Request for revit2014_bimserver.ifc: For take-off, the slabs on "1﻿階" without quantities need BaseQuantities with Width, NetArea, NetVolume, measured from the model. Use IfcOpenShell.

First a look at what the model holds.

```python
import ifcopenshell
import ifcopenshell.util.element
import ifcopenshell.util.unit

model = ifcopenshell.open("revit2014_bimserver.ifc")
print(model.schema)
for unit_type in ("LENGTHUNIT", "AREAUNIT", "VOLUMEUNIT"):
    print(unit_type, ifcopenshell.util.unit.calculate_unit_scale(model, unit_type))
storey = next(s for s in model.by_type("IfcBuildingStorey") if s.Name == '1\ufeff階')
slabs = [e for e in ifcopenshell.util.element.get_decomposition(storey) if e.is_a("IfcSlab")]
for e in sorted(slabs, key=lambda e: e.id()):
    print(e.id(), e.is_a(), e.Name, list(ifcopenshell.util.element.get_psets(e, qtos_only=True)), sep=" | ")
```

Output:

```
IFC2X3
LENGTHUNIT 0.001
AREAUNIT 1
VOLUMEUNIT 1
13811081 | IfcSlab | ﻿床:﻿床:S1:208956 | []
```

```python
import ifcopenshell
import ifcopenshell.api.pset
import ifcopenshell.geom
import ifcopenshell.util.element
import ifcopenshell.util.shape
import ifcopenshell.util.unit

model = ifcopenshell.open("revit2014_bimserver.ifc")
unit_scale = ifcopenshell.util.unit.calculate_unit_scale(model)
area_scale = ifcopenshell.util.unit.calculate_unit_scale(model, "AREAUNIT")
volume_scale = ifcopenshell.util.unit.calculate_unit_scale(model, "VOLUMEUNIT")
settings = ifcopenshell.geom.settings()

storey = next(s for s in model.by_type("IfcBuildingStorey") if s.Name == '1\ufeff階')
slabs = [e for e in ifcopenshell.util.element.get_decomposition(storey) if e.is_a("IfcSlab")]

for e in sorted(slabs, key=lambda e: e.id()):
    if ifcopenshell.util.element.get_psets(e, qtos_only=True, should_inherit=False):
        continue
    # Geometry comes back in metres, in the element's own axes.
    shape = ifcopenshell.geom.create_shape(settings, e)
    values = {
        "Width": ifcopenshell.util.shape.get_z(shape.geometry) / unit_scale,
        "NetArea": ifcopenshell.util.shape.get_footprint_area(shape.geometry) / area_scale,
        "NetVolume": ifcopenshell.util.shape.get_volume(shape.geometry) / volume_scale,
    }
    qto = ifcopenshell.api.pset.add_qto(model, product=e, name="BaseQuantities")
    ifcopenshell.api.pset.edit_qto(model, qto=qto, properties=values)
    print(e.id(), {k: round(v, 3) for k, v in values.items()})

model.write("revit2014_bimserver_edited.ifc")
```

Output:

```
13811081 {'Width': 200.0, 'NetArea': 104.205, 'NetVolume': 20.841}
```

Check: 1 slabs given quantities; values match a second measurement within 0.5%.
